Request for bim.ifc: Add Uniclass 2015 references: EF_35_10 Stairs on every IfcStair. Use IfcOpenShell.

First a look at what the model holds.

```python
import ifcopenshell

model = ifcopenshell.open("bim.ifc")
print(model.schema)
print("classifications:", [c.Name for c in model.by_type("IfcClassification")])
for ifc_class in ("IfcDoor", "IfcRoof", "IfcStair", "IfcWall", "IfcWindow"):
    print(ifc_class, len(model.by_type(ifc_class)))
```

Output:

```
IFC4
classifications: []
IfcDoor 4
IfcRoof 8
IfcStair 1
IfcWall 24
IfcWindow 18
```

```python
import ifcopenshell
import ifcopenshell.api.classification

model = ifcopenshell.open("bim.ifc")

system = ifcopenshell.api.classification.add_classification(model, classification="Uniclass 2015")

codes = {
    "IfcStair": ("EF_35_10", "Stairs"),
}
for ifc_class, (code, name) in codes.items():
    products = model.by_type(ifc_class)
    ifcopenshell.api.classification.add_reference(
        model, products=products, classification=system, identification=code, name=name
    )
    print(code, len(products))

model.write("bim_edited.ifc")
```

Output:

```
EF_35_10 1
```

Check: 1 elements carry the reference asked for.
